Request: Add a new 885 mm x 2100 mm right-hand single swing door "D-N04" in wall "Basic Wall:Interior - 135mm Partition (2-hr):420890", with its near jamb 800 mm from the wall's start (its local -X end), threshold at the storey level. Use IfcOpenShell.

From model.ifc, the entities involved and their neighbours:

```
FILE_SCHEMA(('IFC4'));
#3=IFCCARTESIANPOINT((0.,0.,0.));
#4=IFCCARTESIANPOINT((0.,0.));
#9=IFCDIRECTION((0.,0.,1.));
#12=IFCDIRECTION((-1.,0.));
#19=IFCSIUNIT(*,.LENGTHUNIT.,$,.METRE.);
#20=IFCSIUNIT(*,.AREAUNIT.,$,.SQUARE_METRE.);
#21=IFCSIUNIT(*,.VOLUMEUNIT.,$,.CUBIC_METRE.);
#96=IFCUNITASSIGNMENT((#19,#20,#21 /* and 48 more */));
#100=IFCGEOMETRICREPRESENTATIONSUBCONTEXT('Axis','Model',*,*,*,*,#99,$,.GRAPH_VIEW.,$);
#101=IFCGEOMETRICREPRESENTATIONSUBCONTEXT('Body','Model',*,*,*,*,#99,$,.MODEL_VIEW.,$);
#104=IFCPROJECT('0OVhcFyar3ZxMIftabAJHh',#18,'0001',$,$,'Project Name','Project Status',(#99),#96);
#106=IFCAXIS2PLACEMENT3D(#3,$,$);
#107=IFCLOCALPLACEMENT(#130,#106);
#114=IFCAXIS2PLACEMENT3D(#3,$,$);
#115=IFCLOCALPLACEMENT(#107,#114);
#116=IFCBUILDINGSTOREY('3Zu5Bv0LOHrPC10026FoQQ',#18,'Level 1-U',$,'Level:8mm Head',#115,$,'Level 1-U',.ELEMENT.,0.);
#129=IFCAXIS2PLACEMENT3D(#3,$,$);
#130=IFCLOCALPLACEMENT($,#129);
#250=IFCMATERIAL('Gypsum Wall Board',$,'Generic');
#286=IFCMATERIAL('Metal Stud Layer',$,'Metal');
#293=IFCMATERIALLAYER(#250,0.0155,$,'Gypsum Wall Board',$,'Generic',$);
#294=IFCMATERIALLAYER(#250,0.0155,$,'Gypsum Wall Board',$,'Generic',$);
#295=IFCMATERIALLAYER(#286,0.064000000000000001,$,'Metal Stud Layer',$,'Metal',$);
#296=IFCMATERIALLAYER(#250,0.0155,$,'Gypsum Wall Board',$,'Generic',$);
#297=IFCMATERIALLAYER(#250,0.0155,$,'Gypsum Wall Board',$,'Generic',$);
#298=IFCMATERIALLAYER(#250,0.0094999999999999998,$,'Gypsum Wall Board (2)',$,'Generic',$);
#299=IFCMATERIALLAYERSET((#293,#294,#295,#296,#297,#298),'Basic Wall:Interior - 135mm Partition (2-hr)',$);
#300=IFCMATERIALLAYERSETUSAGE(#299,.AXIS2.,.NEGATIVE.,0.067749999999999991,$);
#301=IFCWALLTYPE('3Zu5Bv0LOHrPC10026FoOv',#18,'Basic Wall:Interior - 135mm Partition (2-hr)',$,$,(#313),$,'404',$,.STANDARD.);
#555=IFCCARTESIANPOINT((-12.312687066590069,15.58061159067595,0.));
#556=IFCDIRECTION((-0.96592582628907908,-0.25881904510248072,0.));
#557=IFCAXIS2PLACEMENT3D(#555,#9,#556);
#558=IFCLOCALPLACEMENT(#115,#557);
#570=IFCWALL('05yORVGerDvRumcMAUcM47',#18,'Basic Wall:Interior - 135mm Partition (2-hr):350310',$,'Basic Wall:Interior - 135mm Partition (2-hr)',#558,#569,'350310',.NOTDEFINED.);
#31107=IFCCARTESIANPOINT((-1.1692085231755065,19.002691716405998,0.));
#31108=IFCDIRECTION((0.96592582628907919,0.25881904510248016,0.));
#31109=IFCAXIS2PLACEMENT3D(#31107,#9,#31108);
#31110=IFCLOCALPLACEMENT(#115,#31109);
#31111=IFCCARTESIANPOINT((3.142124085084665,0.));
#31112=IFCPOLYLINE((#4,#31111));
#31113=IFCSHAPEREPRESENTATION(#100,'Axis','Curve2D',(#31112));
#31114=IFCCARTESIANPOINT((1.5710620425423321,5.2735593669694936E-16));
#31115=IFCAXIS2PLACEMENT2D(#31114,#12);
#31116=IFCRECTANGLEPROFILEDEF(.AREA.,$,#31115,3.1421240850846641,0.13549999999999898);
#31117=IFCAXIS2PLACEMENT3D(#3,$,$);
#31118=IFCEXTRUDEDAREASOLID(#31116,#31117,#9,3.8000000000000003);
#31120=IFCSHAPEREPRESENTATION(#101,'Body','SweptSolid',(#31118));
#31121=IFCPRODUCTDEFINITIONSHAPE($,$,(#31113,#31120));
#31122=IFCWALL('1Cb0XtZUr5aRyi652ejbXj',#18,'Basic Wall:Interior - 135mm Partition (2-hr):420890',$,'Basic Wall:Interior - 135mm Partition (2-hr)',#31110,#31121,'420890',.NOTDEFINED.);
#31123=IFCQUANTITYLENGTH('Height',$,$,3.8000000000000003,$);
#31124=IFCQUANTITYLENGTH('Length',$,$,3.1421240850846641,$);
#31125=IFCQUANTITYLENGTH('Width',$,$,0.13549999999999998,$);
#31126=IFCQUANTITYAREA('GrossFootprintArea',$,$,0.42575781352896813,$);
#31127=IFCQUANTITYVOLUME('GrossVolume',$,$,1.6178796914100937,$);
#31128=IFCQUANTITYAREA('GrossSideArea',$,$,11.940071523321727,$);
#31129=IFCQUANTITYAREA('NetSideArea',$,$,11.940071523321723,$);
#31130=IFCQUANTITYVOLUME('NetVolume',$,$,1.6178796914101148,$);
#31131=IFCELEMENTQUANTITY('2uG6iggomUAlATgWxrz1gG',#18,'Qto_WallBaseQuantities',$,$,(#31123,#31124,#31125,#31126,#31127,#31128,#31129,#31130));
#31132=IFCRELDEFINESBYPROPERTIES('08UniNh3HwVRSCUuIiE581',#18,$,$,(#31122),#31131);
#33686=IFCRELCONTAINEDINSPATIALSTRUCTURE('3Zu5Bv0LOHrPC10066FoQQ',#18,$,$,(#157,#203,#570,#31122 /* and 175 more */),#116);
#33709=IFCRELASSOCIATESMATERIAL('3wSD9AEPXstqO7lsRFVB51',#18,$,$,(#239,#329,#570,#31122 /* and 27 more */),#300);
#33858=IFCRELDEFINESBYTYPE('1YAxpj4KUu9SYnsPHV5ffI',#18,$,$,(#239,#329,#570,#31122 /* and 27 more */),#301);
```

```python
import numpy as np
import ifcopenshell
import ifcopenshell.api.feature
import ifcopenshell.api.geometry
import ifcopenshell.api.pset
import ifcopenshell.api.root
import ifcopenshell.api.spatial
import ifcopenshell.geom
import ifcopenshell.util.element
import ifcopenshell.util.placement
import ifcopenshell.util.representation
import ifcopenshell.util.shape
import ifcopenshell.util.unit

model = ifcopenshell.open("model.ifc")
unit_scale = ifcopenshell.util.unit.calculate_unit_scale(model)
area_scale = ifcopenshell.util.unit.calculate_unit_scale(model, "AREAUNIT")
volume_scale = ifcopenshell.util.unit.calculate_unit_scale(model, "VOLUMEUNIT")
settings = ifcopenshell.geom.settings()


def volume(element):
    """Net volume in cubic metres, openings subtracted."""
    shape = ifcopenshell.geom.create_shape(settings, element)
    return ifcopenshell.util.shape.get_volume(shape.geometry)


wall = model.by_id(31122)
storey = ifcopenshell.util.element.get_container(wall, ifc_class="IfcBuildingStorey")
context = ifcopenshell.util.representation.get_context(model, "Model", "Body", "MODEL_VIEW")
before = volume(wall)

width, height, from_end, sill = 0.885, 2.1, 0.8, 0.0  # metres

# The wall runs along its own X axis, and the end named is its -X end.
wall_shape = ifcopenshell.geom.create_shape(settings, wall)
x, y, z = ifcopenshell.util.shape.get_vertices(wall_shape.geometry).T
start = x.min() + from_end
face, thickness = float(y.min()), float(y.max() - y.min())
wall_matrix = ifcopenshell.util.placement.get_local_placement(wall.ObjectPlacement)
level = ifcopenshell.util.placement.get_local_placement(storey.ObjectPlacement)[2, 3]


def in_wall(x, y):
    """Placement at x, y metres in the wall's axes, at sill height."""
    matrix = wall_matrix.copy()
    matrix[:, 3] = wall_matrix @ np.array([x / unit_scale, y / unit_scale, 0.0, 1.0])
    matrix[2, 3] = level + sill / unit_scale
    return matrix


# Opening: a box that overshoots both wall faces by 50 mm.
opening = ifcopenshell.api.root.create_entity(model, ifc_class="IfcOpeningElement", predefined_type="OPENING")
box = ifcopenshell.api.geometry.add_wall_representation(
    model, context=context, length=width, height=height, thickness=thickness + 0.1
)
ifcopenshell.api.geometry.assign_representation(model, product=opening, representation=box)
ifcopenshell.api.geometry.edit_object_placement(model, product=opening, matrix=in_wall(start, face - 0.05), is_si=False)
ifcopenshell.api.feature.add_feature(model, feature=opening, element=wall)

door = ifcopenshell.api.root.create_entity(model, ifc_class="IfcDoor", name="D-N04", predefined_type="DOOR")
door.OverallWidth, door.OverallHeight = width / unit_scale, height / unit_scale
door.OperationType = "SINGLE_SWING_RIGHT"
body = ifcopenshell.api.geometry.add_door_representation(
    model,
    context=context,
    overall_width=door.OverallWidth,
    overall_height=door.OverallHeight,
    operation_type="SINGLE_SWING_RIGHT",
    lining_properties={"LiningDepth": thickness / unit_scale, "ThresholdDepth": thickness / unit_scale},
)
ifcopenshell.api.geometry.assign_representation(model, product=door, representation=body)
ifcopenshell.api.spatial.assign_container(model, products=[door], relating_structure=storey)
ifcopenshell.api.feature.add_filling(model, opening=opening, element=door)

# The lining spans the wall, so the door starts at the wall face.
ifcopenshell.api.geometry.edit_object_placement(model, product=door, matrix=in_wall(start, face), is_si=False)

after = volume(wall)

# Update the wall's stored quantities.
qto = model.by_id(ifcopenshell.util.element.get_pset(wall, "Qto_WallBaseQuantities", should_inherit=False)["id"])
ifcopenshell.api.pset.edit_qto(model, qto=qto, properties={
    "NetSideArea": after / thickness / area_scale,
    "NetVolume": after / volume_scale,
})

print(f"wall volume {before:.3f} -> {after:.3f} m3")

model.write("model_updated.ifc")
```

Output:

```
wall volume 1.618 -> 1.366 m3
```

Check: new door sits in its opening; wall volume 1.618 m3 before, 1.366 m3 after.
